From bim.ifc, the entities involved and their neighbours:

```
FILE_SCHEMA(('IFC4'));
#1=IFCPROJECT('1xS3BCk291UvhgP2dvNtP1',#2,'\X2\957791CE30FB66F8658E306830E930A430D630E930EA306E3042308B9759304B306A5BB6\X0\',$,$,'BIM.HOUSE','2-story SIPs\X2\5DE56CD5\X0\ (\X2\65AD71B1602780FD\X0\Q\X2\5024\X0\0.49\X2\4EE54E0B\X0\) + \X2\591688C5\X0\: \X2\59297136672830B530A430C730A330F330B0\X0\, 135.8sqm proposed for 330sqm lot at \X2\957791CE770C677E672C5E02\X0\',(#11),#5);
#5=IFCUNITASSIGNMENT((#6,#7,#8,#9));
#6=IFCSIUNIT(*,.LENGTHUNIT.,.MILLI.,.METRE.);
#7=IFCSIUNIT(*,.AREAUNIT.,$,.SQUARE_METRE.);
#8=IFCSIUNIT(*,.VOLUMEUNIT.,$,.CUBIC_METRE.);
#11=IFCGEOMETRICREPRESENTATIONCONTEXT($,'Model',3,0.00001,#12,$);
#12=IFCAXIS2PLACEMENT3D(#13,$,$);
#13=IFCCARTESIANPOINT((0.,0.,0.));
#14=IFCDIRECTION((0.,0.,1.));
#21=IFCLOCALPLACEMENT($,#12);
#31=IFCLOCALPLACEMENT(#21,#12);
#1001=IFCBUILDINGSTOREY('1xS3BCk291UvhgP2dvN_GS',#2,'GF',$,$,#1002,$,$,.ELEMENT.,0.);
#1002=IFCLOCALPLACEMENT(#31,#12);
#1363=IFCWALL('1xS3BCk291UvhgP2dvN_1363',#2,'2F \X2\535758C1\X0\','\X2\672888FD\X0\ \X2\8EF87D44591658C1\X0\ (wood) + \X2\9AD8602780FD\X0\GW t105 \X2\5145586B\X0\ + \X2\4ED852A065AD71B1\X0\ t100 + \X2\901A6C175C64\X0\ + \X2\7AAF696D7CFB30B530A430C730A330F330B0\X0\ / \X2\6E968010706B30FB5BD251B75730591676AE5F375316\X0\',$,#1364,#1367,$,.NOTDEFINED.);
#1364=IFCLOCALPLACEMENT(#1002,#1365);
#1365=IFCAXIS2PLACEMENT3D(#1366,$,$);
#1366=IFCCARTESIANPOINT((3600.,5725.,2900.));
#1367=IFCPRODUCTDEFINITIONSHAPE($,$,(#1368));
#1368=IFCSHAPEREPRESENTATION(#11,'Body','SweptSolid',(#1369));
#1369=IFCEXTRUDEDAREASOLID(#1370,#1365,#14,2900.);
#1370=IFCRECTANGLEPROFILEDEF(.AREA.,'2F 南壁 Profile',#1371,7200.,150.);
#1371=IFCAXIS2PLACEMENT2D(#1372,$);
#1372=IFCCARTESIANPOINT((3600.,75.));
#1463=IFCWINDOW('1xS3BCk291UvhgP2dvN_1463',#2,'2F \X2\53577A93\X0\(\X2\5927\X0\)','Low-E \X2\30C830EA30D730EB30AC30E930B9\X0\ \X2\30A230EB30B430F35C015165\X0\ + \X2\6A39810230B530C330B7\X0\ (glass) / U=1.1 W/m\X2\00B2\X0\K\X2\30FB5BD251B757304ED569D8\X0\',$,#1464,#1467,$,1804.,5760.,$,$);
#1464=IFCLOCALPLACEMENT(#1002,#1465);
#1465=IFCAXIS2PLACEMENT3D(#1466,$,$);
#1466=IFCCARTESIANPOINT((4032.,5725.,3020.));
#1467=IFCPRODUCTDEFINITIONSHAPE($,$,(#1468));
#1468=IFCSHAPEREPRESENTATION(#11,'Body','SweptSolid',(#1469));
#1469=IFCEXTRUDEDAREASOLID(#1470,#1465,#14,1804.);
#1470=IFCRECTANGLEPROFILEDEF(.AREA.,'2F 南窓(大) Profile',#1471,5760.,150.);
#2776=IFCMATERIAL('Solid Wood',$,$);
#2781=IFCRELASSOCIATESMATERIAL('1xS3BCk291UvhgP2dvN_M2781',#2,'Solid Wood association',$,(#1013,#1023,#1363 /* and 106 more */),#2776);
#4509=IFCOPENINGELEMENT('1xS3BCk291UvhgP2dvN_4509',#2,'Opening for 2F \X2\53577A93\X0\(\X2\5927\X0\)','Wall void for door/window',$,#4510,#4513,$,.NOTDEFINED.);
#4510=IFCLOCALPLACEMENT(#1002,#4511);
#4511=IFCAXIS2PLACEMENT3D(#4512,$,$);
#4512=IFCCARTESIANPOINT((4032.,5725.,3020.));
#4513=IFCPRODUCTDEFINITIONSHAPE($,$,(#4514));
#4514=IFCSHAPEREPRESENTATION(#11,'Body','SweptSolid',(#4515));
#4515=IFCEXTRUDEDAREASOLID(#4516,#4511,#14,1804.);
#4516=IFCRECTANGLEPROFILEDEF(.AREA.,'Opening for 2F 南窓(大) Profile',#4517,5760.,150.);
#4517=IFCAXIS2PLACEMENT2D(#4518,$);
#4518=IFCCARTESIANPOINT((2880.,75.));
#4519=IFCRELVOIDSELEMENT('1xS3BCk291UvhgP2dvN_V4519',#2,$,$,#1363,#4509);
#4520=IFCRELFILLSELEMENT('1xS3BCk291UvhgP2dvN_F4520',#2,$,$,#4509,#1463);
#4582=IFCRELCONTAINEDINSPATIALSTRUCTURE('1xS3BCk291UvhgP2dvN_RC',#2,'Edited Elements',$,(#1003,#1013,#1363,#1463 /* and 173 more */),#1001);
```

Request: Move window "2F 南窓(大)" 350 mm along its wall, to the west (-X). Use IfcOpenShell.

```python
import ifcopenshell
import ifcopenshell.api.geometry
import ifcopenshell.util.placement
import ifcopenshell.util.unit

model = ifcopenshell.open("bim.ifc")
unit_scale = ifcopenshell.util.unit.calculate_unit_scale(model)

window = model.by_guid("1xS3BCk291UvhgP2dvN_1463")
opening = window.FillsVoids[0].RelatingOpeningElement
wall = opening.VoidsElements[0].RelatingBuildingElement

wall_matrix = ifcopenshell.util.placement.get_local_placement(wall.ObjectPlacement)
shift = wall_matrix[:3, 0] * -0.35 / unit_scale
before = ifcopenshell.util.placement.get_local_placement(window.ObjectPlacement)[:3, 3].copy()

# The window is not placed relative to its opening, so move both.
for product in (opening, window):
    matrix = ifcopenshell.util.placement.get_local_placement(product.ObjectPlacement)
    matrix[:3, 3] += shift
    ifcopenshell.api.geometry.edit_object_placement(model, product=product, matrix=matrix, is_si=False)

after = ifcopenshell.util.placement.get_local_placement(window.ObjectPlacement)[:3, 3]
print("window moved by", (after - before).round(3) + 0.0)

model.write("bim_updated.ifc")
```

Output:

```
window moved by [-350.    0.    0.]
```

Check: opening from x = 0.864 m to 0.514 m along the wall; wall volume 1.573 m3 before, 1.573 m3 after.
